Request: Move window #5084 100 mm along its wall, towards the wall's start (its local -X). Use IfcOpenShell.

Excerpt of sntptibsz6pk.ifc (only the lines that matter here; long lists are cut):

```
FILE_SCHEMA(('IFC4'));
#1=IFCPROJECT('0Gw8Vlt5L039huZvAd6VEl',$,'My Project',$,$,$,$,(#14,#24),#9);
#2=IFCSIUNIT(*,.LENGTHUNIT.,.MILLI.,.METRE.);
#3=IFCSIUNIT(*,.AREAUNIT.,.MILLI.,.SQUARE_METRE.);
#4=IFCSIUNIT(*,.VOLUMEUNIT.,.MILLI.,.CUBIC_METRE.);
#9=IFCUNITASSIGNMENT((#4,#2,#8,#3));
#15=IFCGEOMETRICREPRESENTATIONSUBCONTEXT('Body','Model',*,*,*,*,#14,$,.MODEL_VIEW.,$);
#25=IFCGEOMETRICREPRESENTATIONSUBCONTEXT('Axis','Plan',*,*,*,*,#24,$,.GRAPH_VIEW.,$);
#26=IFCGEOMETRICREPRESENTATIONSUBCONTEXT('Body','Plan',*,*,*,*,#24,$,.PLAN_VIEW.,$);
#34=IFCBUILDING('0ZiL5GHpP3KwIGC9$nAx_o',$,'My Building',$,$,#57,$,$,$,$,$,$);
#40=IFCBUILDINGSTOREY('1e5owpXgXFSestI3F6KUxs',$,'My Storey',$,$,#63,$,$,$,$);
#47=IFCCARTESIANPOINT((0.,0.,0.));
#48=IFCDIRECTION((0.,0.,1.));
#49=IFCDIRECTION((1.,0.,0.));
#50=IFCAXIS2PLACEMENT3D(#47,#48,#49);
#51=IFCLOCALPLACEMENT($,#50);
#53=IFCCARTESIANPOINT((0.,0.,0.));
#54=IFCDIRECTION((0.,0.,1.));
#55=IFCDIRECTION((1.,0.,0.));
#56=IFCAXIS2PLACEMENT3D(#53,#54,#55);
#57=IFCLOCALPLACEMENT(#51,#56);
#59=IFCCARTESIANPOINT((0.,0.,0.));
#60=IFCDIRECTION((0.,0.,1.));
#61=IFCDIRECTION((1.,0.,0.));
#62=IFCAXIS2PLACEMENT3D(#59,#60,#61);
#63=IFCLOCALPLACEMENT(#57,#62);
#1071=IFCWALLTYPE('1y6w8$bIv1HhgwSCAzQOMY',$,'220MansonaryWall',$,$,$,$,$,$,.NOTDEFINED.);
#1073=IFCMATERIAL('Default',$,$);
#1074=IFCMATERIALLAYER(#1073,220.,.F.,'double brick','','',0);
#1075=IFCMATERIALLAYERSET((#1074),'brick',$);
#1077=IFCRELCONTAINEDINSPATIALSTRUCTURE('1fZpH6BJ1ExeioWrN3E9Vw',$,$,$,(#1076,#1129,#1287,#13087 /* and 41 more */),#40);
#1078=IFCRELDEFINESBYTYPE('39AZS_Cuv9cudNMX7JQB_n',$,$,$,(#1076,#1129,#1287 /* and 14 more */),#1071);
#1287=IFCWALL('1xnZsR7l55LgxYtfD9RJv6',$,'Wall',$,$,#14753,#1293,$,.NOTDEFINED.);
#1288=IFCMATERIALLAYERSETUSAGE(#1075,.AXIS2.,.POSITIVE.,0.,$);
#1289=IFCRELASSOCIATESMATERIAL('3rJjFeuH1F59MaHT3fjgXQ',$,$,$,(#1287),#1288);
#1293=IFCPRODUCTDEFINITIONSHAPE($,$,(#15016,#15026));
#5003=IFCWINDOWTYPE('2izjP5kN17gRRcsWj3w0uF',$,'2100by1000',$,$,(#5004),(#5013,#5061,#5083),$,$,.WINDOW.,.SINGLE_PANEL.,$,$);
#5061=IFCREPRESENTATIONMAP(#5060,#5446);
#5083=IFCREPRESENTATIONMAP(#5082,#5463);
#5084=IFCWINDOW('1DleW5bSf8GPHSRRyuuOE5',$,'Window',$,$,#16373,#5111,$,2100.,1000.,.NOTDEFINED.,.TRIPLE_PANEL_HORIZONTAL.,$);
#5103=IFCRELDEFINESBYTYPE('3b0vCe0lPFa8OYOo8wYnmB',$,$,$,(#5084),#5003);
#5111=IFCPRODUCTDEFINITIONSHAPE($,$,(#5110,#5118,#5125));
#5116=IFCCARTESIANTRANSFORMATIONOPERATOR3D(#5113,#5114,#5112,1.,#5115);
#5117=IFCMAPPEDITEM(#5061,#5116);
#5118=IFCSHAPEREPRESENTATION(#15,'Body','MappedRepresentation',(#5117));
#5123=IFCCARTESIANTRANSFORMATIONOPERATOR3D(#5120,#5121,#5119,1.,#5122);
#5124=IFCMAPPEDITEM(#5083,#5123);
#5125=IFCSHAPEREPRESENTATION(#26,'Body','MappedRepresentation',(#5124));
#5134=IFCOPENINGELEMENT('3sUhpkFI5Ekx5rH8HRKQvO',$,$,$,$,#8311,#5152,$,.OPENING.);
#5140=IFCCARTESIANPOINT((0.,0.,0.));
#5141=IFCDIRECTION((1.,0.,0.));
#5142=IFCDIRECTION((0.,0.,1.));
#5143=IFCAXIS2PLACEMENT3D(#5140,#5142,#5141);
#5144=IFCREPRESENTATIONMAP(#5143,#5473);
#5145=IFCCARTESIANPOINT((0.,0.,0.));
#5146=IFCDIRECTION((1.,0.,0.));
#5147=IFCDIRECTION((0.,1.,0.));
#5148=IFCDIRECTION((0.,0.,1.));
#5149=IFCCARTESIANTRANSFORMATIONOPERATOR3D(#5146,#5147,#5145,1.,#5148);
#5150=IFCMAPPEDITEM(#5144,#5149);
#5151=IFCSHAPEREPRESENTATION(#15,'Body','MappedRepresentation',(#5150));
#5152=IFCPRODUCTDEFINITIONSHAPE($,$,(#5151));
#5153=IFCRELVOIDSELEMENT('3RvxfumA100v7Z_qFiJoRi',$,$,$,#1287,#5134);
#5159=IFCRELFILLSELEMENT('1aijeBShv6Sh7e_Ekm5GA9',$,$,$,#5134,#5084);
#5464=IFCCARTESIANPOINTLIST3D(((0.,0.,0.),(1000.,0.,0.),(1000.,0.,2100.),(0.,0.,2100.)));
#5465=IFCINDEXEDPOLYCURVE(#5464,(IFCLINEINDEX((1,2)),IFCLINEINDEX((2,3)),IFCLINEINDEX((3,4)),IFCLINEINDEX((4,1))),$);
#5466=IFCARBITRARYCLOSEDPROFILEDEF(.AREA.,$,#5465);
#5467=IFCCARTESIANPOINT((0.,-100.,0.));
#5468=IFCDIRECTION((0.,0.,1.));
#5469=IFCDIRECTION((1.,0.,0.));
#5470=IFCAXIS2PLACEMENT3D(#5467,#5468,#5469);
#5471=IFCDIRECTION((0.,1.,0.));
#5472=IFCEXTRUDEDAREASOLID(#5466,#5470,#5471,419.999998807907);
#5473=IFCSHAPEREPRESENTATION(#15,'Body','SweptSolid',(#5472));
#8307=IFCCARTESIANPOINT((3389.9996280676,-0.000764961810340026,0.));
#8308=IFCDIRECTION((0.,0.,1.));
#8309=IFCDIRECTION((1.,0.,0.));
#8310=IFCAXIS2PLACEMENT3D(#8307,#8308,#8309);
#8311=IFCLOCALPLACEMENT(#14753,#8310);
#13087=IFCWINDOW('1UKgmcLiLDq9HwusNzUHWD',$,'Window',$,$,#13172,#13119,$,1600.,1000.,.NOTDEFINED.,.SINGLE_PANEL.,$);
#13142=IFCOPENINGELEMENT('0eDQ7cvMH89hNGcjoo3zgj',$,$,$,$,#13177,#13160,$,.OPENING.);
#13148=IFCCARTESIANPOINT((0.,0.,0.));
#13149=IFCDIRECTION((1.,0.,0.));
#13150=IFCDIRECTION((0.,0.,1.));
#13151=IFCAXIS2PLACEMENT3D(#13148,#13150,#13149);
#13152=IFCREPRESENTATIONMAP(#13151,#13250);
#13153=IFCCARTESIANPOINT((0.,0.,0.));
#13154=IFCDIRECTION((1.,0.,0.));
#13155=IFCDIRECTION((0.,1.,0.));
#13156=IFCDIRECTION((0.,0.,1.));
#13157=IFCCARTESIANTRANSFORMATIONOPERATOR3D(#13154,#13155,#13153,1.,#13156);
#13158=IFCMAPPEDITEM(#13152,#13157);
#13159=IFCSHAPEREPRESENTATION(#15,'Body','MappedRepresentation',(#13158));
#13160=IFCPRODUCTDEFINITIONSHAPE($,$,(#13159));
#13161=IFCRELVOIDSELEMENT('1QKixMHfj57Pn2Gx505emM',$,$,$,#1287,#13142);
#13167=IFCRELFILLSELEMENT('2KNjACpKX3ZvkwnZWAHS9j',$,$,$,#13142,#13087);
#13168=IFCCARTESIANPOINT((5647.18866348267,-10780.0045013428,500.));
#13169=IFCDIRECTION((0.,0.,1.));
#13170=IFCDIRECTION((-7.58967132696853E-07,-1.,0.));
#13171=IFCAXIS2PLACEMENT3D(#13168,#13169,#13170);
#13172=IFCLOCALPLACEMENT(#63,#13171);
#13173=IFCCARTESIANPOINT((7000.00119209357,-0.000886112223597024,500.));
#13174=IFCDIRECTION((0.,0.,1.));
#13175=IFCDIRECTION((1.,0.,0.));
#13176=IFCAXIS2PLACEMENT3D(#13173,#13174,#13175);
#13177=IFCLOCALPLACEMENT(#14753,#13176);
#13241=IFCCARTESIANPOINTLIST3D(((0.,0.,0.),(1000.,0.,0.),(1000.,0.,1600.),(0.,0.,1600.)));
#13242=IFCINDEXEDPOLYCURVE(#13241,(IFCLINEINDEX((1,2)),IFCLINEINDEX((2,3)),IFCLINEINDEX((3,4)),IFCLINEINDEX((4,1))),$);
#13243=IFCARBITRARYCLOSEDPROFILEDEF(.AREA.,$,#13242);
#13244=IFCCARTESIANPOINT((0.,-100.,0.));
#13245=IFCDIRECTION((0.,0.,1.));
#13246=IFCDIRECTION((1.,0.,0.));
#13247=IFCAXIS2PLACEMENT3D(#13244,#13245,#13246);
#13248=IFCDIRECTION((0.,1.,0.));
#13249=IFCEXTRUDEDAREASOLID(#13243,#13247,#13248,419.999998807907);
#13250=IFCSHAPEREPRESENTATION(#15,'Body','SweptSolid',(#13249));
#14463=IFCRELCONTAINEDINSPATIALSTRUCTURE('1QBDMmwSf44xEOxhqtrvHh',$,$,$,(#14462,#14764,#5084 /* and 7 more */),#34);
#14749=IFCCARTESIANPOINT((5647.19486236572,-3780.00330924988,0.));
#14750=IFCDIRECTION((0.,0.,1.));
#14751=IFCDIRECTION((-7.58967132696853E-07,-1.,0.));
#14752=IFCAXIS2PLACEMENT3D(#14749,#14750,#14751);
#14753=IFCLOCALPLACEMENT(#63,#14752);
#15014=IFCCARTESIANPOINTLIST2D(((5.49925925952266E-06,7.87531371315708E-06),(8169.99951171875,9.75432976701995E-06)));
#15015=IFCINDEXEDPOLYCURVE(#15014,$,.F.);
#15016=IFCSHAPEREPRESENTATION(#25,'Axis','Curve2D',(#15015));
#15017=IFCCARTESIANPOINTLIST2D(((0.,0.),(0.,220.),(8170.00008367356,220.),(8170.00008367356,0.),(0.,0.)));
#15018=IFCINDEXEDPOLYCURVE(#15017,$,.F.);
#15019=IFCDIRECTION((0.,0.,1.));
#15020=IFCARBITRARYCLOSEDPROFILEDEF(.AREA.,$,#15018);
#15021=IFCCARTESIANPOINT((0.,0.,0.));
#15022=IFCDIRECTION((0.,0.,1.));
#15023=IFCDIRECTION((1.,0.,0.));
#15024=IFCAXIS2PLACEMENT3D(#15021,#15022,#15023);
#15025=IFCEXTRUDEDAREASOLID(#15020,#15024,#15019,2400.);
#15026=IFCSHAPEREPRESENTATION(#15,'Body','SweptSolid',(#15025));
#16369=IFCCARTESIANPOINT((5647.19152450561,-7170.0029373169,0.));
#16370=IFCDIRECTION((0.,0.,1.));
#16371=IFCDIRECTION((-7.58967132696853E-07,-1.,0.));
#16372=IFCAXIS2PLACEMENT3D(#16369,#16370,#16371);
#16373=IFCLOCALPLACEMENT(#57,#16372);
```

```python
import ifcopenshell
import ifcopenshell.api.geometry
import ifcopenshell.util.placement
import ifcopenshell.util.unit

model = ifcopenshell.open("sntptibsz6pk.ifc")
unit_scale = ifcopenshell.util.unit.calculate_unit_scale(model)

window = model.by_guid("1DleW5bSf8GPHSRRyuuOE5")
opening = window.FillsVoids[0].RelatingOpeningElement
wall = opening.VoidsElements[0].RelatingBuildingElement

wall_matrix = ifcopenshell.util.placement.get_local_placement(wall.ObjectPlacement)
shift = wall_matrix[:3, 0] * -0.1 / unit_scale
before = ifcopenshell.util.placement.get_local_placement(window.ObjectPlacement)[:3, 3].copy()

# The window is not placed relative to its opening, so move both.
for product in (opening, window):
    matrix = ifcopenshell.util.placement.get_local_placement(product.ObjectPlacement)
    matrix[:3, 3] += shift
    ifcopenshell.api.geometry.edit_object_placement(model, product=product, matrix=matrix, is_si=False)

after = ifcopenshell.util.placement.get_local_placement(window.ObjectPlacement)[:3, 3]
print("window moved by", (after - before).round(3) + 0.0)

model.write("sntptibsz6pk-out.ifc")
```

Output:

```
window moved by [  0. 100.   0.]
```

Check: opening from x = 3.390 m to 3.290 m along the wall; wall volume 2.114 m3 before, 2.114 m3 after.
